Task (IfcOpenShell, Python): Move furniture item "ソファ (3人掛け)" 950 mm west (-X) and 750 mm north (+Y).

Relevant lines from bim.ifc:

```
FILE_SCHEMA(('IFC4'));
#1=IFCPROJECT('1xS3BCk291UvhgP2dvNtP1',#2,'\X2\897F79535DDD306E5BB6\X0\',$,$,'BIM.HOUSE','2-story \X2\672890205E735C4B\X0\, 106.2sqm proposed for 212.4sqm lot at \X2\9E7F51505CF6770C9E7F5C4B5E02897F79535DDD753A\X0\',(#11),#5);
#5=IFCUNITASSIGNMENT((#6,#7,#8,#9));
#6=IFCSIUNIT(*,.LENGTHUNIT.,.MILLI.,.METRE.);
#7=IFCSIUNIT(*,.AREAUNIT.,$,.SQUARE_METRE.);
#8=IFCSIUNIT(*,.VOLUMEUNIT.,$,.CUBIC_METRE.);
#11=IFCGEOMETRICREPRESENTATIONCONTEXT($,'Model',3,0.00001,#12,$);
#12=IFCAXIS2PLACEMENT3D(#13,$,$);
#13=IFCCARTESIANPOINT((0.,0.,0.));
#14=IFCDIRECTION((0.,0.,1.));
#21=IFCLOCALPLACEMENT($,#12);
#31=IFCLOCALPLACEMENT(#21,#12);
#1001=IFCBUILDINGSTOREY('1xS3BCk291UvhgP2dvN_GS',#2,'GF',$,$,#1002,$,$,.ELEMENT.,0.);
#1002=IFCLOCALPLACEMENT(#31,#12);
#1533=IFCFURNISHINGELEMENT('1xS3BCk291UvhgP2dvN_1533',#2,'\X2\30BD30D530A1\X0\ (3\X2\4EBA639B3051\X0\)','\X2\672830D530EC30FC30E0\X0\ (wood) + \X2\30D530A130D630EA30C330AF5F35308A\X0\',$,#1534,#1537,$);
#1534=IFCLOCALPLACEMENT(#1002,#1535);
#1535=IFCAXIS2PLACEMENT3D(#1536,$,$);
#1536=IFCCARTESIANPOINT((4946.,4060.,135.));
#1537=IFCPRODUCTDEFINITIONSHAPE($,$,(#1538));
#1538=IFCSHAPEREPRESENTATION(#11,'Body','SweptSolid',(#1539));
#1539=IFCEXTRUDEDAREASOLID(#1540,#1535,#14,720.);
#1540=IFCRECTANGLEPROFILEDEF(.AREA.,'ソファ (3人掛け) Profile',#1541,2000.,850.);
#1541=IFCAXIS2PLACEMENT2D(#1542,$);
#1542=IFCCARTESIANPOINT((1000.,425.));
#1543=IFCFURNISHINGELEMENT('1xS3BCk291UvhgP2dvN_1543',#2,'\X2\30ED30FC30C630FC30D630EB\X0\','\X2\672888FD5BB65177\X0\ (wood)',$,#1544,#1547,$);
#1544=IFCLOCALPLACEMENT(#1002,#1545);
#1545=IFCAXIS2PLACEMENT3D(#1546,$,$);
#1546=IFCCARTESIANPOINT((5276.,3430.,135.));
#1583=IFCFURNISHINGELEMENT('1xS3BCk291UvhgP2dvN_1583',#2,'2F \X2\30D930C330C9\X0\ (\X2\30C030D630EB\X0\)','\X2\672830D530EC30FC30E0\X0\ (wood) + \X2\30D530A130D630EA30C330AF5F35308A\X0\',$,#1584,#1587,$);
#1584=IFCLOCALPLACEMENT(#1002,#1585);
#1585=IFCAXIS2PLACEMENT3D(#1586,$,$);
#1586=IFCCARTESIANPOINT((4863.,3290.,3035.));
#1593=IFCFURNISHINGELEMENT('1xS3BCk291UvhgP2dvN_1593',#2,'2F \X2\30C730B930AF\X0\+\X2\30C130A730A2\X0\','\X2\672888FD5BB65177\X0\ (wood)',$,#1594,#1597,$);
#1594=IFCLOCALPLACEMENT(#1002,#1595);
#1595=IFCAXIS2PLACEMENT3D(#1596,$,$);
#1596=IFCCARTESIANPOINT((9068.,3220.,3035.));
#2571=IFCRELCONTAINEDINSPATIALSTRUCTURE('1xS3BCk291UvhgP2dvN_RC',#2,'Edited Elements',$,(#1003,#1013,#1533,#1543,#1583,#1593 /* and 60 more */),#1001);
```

```python
import ifcopenshell
import ifcopenshell.api.geometry
import ifcopenshell.util.placement
import ifcopenshell.util.unit

model = ifcopenshell.open("bim.ifc")
unit_scale = ifcopenshell.util.unit.calculate_unit_scale(model)

item = model.by_guid("1xS3BCk291UvhgP2dvN_1533")
matrix = ifcopenshell.util.placement.get_local_placement(item.ObjectPlacement)
matrix[0, 3] -= 0.95 / unit_scale
matrix[1, 3] += 0.75 / unit_scale
ifcopenshell.api.geometry.edit_object_placement(model, product=item, matrix=matrix, is_si=False)

print(ifcopenshell.util.placement.get_local_placement(item.ObjectPlacement).round(3) + 0.0)

model.write("bim_edited.ifc")
```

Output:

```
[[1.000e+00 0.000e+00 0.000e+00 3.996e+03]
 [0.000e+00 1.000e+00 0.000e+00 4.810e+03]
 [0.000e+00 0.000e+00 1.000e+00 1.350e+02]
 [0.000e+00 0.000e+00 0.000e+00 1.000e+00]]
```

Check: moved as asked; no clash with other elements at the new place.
